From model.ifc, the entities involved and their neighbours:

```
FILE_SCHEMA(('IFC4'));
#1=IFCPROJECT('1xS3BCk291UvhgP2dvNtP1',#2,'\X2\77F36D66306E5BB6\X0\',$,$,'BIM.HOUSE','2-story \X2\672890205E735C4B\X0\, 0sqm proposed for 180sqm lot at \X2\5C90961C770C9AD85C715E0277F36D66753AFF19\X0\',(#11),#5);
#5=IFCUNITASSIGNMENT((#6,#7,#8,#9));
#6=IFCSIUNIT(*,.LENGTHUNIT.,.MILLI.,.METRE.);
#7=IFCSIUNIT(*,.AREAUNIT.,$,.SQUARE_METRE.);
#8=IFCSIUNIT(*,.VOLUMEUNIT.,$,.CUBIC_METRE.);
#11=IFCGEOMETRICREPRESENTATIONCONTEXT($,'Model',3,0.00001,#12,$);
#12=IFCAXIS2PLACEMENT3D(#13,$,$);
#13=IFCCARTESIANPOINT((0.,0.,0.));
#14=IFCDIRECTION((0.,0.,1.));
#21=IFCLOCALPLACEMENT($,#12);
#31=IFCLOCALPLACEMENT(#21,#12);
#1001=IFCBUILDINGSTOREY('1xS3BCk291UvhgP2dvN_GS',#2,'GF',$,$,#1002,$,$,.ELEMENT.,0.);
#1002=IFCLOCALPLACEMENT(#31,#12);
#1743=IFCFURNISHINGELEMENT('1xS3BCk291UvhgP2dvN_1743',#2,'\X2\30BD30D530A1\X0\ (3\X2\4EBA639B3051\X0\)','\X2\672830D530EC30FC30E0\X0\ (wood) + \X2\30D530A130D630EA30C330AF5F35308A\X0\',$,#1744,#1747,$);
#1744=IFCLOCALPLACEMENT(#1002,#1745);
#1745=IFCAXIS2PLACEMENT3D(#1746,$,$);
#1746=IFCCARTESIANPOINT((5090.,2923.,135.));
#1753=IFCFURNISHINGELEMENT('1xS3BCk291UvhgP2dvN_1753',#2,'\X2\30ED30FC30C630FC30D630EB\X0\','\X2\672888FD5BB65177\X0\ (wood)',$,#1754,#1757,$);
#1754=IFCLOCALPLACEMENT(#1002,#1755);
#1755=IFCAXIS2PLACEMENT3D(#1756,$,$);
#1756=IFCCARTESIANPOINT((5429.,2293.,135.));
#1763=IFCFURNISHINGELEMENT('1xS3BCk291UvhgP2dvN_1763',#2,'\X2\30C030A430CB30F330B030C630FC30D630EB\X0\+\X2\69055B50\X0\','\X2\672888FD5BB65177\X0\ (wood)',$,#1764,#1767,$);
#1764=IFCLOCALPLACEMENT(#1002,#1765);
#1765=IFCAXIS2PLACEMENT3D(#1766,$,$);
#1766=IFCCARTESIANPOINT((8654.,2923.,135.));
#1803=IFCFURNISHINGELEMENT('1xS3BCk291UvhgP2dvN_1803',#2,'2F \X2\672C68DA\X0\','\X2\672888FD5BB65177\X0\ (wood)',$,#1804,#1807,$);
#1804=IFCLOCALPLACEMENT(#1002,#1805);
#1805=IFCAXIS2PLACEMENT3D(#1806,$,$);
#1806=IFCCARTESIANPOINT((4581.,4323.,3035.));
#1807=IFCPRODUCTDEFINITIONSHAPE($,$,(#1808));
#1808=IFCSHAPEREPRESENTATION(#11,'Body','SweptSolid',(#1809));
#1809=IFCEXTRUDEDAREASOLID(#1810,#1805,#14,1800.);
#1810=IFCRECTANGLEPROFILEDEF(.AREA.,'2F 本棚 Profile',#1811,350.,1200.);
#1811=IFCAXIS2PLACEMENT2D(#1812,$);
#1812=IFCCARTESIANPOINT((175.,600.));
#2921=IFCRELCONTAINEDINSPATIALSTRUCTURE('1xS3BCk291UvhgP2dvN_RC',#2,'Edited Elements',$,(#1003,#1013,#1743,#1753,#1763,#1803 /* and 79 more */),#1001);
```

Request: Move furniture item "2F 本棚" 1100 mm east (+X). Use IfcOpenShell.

```python
import ifcopenshell
import ifcopenshell.api.geometry
import ifcopenshell.util.placement
import ifcopenshell.util.unit

model = ifcopenshell.open("model.ifc")
unit_scale = ifcopenshell.util.unit.calculate_unit_scale(model)

item = model.by_guid("1xS3BCk291UvhgP2dvN_1803")
matrix = ifcopenshell.util.placement.get_local_placement(item.ObjectPlacement)
matrix[0, 3] += 1.1 / unit_scale
ifcopenshell.api.geometry.edit_object_placement(model, product=item, matrix=matrix, is_si=False)

print(ifcopenshell.util.placement.get_local_placement(item.ObjectPlacement).round(3) + 0.0)

model.write("model_edited.ifc")
```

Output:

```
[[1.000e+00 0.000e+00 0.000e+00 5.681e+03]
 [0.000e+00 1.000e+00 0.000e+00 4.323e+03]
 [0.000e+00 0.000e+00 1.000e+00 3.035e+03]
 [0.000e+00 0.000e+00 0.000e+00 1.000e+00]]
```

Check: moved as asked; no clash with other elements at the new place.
